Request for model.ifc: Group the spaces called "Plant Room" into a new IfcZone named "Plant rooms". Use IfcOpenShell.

First a look at what the model holds.

```python
import ifcopenshell

model = ifcopenshell.open("model.ifc")
print(model.schema)
seen = {}
for space in model.by_type("IfcSpace"):
    seen[space.LongName] = seen.get(space.LongName, 0) + 1
for name, count in sorted(seen.items(), key=str):
    print(count, "x", name)
print("zones:", [z.Name for z in model.by_type("IfcZone")][:20])
```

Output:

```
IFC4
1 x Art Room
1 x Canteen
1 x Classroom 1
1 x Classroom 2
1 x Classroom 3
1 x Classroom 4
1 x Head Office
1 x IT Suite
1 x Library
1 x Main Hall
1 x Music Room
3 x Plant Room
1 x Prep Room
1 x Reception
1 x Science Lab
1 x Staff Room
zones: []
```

```python
import ifcopenshell
import ifcopenshell.api.group
import ifcopenshell.api.root

model = ifcopenshell.open("model.ifc")

names = {"Plant Room"}
spaces = [s for s in model.by_type("IfcSpace") if s.LongName in names]

zone = ifcopenshell.api.root.create_entity(model, ifc_class="IfcZone", name="Plant rooms")
ifcopenshell.api.group.assign_group(model, products=spaces, group=zone)
print(len(spaces), "spaces in", zone.Name)

model.write("model_edited.ifc")
```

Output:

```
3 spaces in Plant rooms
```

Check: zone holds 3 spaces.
